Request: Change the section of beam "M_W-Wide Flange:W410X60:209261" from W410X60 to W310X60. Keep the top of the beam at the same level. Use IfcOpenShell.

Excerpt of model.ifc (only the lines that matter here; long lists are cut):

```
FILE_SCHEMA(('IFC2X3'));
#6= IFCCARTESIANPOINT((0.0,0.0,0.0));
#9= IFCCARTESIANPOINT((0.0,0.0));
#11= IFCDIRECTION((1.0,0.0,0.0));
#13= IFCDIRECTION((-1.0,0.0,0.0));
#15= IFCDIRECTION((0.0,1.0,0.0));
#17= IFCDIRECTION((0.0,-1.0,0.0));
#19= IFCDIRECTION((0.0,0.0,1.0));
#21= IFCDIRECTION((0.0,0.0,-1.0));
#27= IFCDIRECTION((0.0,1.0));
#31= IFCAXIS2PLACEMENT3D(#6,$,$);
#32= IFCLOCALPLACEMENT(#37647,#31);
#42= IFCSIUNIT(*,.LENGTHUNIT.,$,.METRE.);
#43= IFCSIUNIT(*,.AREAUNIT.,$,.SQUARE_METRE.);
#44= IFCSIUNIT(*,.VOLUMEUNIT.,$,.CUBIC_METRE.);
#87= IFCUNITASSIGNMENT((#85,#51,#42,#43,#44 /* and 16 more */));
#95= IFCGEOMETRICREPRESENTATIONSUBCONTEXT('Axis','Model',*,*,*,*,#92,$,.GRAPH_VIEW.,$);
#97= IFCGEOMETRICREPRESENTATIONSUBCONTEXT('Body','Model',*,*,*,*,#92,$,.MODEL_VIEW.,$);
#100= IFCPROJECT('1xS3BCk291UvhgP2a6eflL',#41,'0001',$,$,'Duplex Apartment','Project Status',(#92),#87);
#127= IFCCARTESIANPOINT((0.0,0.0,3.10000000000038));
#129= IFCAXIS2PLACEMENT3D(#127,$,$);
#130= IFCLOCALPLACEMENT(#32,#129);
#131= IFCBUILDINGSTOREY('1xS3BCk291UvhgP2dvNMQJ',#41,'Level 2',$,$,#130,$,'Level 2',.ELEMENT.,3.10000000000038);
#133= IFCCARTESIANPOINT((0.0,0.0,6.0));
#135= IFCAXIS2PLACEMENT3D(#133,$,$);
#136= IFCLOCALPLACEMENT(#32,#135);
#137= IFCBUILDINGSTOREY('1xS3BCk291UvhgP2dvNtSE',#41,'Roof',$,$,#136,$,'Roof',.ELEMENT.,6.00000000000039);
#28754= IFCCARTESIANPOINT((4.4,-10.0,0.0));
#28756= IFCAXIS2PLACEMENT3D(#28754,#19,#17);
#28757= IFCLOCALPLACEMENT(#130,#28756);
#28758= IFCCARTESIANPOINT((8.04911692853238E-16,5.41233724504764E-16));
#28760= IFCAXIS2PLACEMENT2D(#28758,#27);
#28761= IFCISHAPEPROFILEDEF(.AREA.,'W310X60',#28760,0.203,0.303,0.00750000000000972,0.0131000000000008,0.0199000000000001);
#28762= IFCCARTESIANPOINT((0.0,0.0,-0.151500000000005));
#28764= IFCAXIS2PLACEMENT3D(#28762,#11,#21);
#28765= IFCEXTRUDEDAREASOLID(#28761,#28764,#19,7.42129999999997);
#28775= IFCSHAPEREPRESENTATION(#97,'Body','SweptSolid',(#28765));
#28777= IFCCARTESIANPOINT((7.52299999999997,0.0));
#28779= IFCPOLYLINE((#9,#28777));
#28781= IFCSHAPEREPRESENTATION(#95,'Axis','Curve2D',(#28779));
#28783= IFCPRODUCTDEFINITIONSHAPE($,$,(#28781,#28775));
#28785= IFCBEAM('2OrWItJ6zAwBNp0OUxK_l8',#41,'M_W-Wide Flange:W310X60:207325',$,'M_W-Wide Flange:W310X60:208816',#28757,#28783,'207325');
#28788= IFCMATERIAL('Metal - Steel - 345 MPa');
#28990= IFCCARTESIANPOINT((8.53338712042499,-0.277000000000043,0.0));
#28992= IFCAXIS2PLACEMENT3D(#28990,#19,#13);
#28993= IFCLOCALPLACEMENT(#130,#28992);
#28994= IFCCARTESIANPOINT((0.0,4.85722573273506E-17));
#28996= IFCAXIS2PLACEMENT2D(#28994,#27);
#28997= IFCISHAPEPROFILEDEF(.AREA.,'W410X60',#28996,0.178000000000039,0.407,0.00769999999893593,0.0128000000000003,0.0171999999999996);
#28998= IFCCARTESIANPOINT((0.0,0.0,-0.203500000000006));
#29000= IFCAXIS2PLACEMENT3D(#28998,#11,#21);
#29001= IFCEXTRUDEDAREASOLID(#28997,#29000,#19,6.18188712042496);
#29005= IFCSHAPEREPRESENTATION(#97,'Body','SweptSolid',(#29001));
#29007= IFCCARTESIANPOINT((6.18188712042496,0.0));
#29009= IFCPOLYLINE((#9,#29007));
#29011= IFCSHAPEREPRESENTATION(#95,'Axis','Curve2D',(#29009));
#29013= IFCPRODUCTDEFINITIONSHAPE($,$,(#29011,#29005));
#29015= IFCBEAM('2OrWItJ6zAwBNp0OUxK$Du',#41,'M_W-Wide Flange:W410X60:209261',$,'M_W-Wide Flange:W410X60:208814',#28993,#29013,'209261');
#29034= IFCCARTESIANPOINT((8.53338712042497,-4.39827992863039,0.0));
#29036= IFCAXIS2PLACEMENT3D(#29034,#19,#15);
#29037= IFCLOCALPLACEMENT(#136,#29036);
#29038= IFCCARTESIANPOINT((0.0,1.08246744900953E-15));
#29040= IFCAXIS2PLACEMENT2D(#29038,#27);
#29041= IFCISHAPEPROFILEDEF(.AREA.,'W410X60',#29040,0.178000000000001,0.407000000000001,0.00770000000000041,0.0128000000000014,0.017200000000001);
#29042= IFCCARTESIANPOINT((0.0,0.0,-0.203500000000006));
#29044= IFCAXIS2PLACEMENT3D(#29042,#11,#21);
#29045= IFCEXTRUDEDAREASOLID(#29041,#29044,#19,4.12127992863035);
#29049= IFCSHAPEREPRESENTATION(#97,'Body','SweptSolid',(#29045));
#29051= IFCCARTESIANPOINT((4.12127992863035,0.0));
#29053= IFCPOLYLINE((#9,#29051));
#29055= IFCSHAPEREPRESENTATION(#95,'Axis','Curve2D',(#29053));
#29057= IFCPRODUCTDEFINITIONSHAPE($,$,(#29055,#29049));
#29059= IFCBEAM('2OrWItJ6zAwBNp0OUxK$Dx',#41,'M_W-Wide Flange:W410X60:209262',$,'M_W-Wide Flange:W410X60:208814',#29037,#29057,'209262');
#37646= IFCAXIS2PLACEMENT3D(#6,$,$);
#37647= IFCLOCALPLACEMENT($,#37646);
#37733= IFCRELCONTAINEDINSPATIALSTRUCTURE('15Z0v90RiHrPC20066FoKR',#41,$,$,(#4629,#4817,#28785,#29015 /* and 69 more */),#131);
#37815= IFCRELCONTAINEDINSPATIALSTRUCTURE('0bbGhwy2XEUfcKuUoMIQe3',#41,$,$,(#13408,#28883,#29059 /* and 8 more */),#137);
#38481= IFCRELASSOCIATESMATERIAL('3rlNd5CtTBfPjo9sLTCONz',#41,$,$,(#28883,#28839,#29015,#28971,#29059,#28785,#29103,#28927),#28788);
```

```python
import ifcopenshell
import ifcopenshell.util.element
import ifcopenshell.util.representation

model = ifcopenshell.open("model.ifc")

member = model.by_guid("2OrWItJ6zAwBNp0OUxK$Du")
source = next(p for p in model.by_type("IfcIShapeProfileDef") if p.ProfileName == "W310X60")

body = ifcopenshell.util.representation.get_representation(member, "Model", "Body")
solid = body.Items[0]
old_profile = solid.SweptArea

# Copy the section's sizes but keep this member's own profile position.
profile = ifcopenshell.util.element.copy(model, source)
# Profiles are centred, so shift by half the change in depth to hold the top.
shift = (old_profile.OverallDepth - profile.OverallDepth) / 2
x, y = old_profile.Position.Location.Coordinates
up = (-1.0, 0.0)  # upwards, in the solid's own plane
location = model.createIfcCartesianPoint((x + up[0] * shift, y + up[1] * shift))
profile.Position = model.createIfcAxis2Placement2D(location, old_profile.Position.RefDirection)
solid.SweptArea = profile
if not model.get_total_inverses(old_profile):
    ifcopenshell.util.element.remove_deep2(model, old_profile)
member.Name = member.Name.replace("W410X60", "W310X60")
member.ObjectType = member.ObjectType.replace("W410X60", "W310X60")

print(solid.SweptArea)

model.write("model-out.ifc")
```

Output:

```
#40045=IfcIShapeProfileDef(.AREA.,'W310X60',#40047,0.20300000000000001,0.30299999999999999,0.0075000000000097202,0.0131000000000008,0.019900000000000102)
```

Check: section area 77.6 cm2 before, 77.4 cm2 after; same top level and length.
